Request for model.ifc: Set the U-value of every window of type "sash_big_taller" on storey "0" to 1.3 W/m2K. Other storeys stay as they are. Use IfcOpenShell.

First a look at what the model holds.

```python
import ifcopenshell
import ifcopenshell.util.element

model = ifcopenshell.open("model.ifc")
print(model.schema)
storey = next(s for s in model.by_type("IfcBuildingStorey") if s.Name == "0")
windows = [e for e in ifcopenshell.util.element.get_decomposition(storey) if e.is_a("IfcWindow")]
seen = {}
for e in windows:
    element_type = ifcopenshell.util.element.get_type(e)
    key = (element_type.Name if element_type != e and element_type else None, ifcopenshell.util.element.get_pset(e, "Pset_WindowCommon", "ThermalTransmittance"))
    seen[key] = seen.get(key, 0) + 1
for (name, value), count in sorted(seen.items(), key=str):
    print(count, "x", name, "|", value)
```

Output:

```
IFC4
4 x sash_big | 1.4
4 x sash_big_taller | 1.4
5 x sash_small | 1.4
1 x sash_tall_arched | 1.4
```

```python
import ifcopenshell
import ifcopenshell.api.pset
import ifcopenshell.util.element

model = ifcopenshell.open("model.ifc")

storey = next(s for s in model.by_type("IfcBuildingStorey") if s.Name == "0")
windows = [e for e in ifcopenshell.util.element.get_decomposition(storey) if e.is_a("IfcWindow")]

count = 0
for e in windows:
    element_type = ifcopenshell.util.element.get_type(e)
    if element_type in (None, e) or element_type.Name != "sash_big_taller":
        continue
    # add_pset returns the element's existing set when there is one.
    pset = ifcopenshell.api.pset.add_pset(model, product=e, name="Pset_WindowCommon")
    ifcopenshell.api.pset.edit_pset(model, pset=pset, properties={"ThermalTransmittance": 1.3})
    count += 1

print(count, "windows updated")

model.write("model_rev.ifc")
```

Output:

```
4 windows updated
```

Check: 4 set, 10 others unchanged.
